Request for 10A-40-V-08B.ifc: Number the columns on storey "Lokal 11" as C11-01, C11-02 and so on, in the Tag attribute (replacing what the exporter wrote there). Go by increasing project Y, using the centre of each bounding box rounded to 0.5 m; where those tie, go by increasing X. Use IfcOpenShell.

First a look at what the model holds.

```python
import ifcopenshell
import ifcopenshell.util.element
import ifcopenshell.util.placement

model = ifcopenshell.open("10A-40-V-08B.ifc")
print(model.schema)
storey = next(s for s in model.by_type("IfcBuildingStorey") if s.Name == "Lokal 11")
columns = [e for e in ifcopenshell.util.element.get_decomposition(storey) if e.is_a("IfcColumn")]
for e in sorted(columns, key=lambda e: e.id()):
    origin = ifcopenshell.util.placement.get_local_placement(e.ObjectPlacement)[:3, 3]
    print(e.id(), e.Tag, e.Name, origin.round(2) + 0.0, sep=" | ")
```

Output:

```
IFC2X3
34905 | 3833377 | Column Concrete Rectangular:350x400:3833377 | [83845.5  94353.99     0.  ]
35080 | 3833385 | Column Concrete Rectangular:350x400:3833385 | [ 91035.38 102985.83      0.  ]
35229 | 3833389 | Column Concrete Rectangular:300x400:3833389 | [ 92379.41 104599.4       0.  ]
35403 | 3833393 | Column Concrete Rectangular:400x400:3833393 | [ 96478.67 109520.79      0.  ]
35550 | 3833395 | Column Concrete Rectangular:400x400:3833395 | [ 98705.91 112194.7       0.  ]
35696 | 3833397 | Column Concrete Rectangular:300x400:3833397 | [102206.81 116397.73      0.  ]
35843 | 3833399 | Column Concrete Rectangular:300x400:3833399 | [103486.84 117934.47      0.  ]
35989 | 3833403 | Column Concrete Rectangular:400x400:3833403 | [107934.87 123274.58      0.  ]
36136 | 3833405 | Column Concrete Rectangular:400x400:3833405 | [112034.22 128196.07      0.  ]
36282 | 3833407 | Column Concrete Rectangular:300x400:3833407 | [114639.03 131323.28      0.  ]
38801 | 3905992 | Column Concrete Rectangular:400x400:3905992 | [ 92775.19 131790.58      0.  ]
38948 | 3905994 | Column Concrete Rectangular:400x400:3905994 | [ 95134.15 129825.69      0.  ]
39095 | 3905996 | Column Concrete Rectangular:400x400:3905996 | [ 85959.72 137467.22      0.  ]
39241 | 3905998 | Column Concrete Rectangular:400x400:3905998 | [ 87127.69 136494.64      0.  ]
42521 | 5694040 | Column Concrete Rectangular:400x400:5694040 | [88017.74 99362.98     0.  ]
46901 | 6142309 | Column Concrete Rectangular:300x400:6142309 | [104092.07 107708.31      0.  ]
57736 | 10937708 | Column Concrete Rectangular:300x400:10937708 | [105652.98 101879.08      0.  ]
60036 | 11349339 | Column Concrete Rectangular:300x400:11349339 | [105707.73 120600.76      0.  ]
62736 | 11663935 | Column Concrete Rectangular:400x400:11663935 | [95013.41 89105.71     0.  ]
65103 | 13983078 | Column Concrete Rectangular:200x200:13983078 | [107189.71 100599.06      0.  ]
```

```python
import ifcopenshell
import ifcopenshell.geom
import ifcopenshell.util.element
import ifcopenshell.util.shape

model = ifcopenshell.open("10A-40-V-08B.ifc")
settings = ifcopenshell.geom.settings()
settings.set("use-world-coords", True)


def centre(element):
    shape = ifcopenshell.geom.create_shape(settings, element)
    return ifcopenshell.util.shape.get_bbox_centroid(shape.geometry)


storey = next(s for s in model.by_type("IfcBuildingStorey") if s.Name == "Lokal 11")
columns = [e for e in ifcopenshell.util.element.get_decomposition(storey) if e.is_a("IfcColumn")]

# Insertion points can sit at a corner or the storey origin, so sort by the geometry (in metres).
centres = {e: centre(e) for e in columns}
columns.sort(key=lambda e: (round(centres[e][1] / 0.5), centres[e][0]))

for i, e in enumerate(columns, start=1):
    number = f"C11-{i:02d}"
    e.Tag = number
    print(e.id(), number)

model.write("10A-40-V-08B_edited.ifc")
```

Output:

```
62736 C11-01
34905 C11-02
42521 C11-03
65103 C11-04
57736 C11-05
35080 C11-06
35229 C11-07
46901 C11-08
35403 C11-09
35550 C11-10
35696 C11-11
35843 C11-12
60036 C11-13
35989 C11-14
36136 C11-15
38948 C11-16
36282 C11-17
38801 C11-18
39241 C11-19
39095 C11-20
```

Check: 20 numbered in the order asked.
